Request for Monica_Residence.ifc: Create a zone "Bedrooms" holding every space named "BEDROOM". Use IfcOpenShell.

First a look at what the model holds.

```python
import ifcopenshell

model = ifcopenshell.open("Monica_Residence.ifc")
print(model.schema)
seen = {}
for space in model.by_type("IfcSpace"):
    seen[space.LongName] = seen.get(space.LongName, 0) + 1
for name, count in sorted(seen.items(), key=str):
    print(count, "x", name)
print("zones:", [z.Name for z in model.by_type("IfcZone")][:20])
```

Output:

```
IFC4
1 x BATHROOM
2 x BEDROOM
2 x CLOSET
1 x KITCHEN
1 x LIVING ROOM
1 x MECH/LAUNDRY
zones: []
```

```python
import ifcopenshell
import ifcopenshell.api.group
import ifcopenshell.api.root

model = ifcopenshell.open("Monica_Residence.ifc")

names = {"BEDROOM"}
spaces = [s for s in model.by_type("IfcSpace") if s.LongName in names]

zone = ifcopenshell.api.root.create_entity(model, ifc_class="IfcZone", name="Bedrooms")
ifcopenshell.api.group.assign_group(model, products=spaces, group=zone)
print(len(spaces), "spaces in", zone.Name)

model.write("Monica_Residence_edited.ifc")
```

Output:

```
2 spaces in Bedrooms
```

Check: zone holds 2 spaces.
